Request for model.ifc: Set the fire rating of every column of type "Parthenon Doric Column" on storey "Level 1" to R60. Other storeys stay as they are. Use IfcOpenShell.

First a look at what the model holds.

```python
import ifcopenshell
import ifcopenshell.util.element

model = ifcopenshell.open("model.ifc")
print(model.schema)
storey = next(s for s in model.by_type("IfcBuildingStorey") if s.Name == "Level 1")
columns = [e for e in ifcopenshell.util.element.get_decomposition(storey) if e.is_a("IfcColumn")]
seen = {}
for e in columns:
    element_type = ifcopenshell.util.element.get_type(e)
    key = (element_type.Name if element_type != e and element_type else None, ifcopenshell.util.element.get_pset(e, "Pset_ColumnCommon", "FireRating"))
    seen[key] = seen.get(key, 0) + 1
for (name, value), count in sorted(seen.items(), key=str):
    print(count, "x", name, "|", value)
```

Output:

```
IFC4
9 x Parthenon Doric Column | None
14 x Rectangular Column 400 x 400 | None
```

```python
import ifcopenshell
import ifcopenshell.api.pset
import ifcopenshell.util.element

model = ifcopenshell.open("model.ifc")

storey = next(s for s in model.by_type("IfcBuildingStorey") if s.Name == "Level 1")
columns = [e for e in ifcopenshell.util.element.get_decomposition(storey) if e.is_a("IfcColumn")]

count = 0
for e in columns:
    element_type = ifcopenshell.util.element.get_type(e)
    if element_type in (None, e) or element_type.Name != "Parthenon Doric Column":
        continue
    # add_pset returns the element's existing set when there is one.
    pset = ifcopenshell.api.pset.add_pset(model, product=e, name="Pset_ColumnCommon")
    ifcopenshell.api.pset.edit_pset(model, pset=pset, properties={"FireRating": "R60"})
    count += 1

print(count, "columns updated")

model.write("model-out.ifc")
```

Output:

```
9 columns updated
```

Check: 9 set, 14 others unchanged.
